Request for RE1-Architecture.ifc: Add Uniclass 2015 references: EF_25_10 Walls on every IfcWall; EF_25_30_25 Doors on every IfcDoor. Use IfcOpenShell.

First a look at what the model holds.

```python
import ifcopenshell

model = ifcopenshell.open("RE1-Architecture.ifc")
print(model.schema)
print("classifications:", [c.Name for c in model.by_type("IfcClassification")])
for ifc_class in ("IfcDoor", "IfcRoof", "IfcStair", "IfcWall", "IfcWindow"):
    print(ifc_class, len(model.by_type(ifc_class)))
```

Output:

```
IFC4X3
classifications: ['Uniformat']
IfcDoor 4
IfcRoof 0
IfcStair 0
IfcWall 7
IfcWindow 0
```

```python
import ifcopenshell
import ifcopenshell.api.classification

model = ifcopenshell.open("RE1-Architecture.ifc")

system = ifcopenshell.api.classification.add_classification(model, classification="Uniclass 2015")

codes = {
    "IfcWall": ("EF_25_10", "Walls"),
    "IfcDoor": ("EF_25_30_25", "Doors"),
}
for ifc_class, (code, name) in codes.items():
    products = model.by_type(ifc_class)
    ifcopenshell.api.classification.add_reference(
        model, products=products, classification=system, identification=code, name=name
    )
    print(code, len(products))

model.write("RE1-Architecture_rev.ifc")
```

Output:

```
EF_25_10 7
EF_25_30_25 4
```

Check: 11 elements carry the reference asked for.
